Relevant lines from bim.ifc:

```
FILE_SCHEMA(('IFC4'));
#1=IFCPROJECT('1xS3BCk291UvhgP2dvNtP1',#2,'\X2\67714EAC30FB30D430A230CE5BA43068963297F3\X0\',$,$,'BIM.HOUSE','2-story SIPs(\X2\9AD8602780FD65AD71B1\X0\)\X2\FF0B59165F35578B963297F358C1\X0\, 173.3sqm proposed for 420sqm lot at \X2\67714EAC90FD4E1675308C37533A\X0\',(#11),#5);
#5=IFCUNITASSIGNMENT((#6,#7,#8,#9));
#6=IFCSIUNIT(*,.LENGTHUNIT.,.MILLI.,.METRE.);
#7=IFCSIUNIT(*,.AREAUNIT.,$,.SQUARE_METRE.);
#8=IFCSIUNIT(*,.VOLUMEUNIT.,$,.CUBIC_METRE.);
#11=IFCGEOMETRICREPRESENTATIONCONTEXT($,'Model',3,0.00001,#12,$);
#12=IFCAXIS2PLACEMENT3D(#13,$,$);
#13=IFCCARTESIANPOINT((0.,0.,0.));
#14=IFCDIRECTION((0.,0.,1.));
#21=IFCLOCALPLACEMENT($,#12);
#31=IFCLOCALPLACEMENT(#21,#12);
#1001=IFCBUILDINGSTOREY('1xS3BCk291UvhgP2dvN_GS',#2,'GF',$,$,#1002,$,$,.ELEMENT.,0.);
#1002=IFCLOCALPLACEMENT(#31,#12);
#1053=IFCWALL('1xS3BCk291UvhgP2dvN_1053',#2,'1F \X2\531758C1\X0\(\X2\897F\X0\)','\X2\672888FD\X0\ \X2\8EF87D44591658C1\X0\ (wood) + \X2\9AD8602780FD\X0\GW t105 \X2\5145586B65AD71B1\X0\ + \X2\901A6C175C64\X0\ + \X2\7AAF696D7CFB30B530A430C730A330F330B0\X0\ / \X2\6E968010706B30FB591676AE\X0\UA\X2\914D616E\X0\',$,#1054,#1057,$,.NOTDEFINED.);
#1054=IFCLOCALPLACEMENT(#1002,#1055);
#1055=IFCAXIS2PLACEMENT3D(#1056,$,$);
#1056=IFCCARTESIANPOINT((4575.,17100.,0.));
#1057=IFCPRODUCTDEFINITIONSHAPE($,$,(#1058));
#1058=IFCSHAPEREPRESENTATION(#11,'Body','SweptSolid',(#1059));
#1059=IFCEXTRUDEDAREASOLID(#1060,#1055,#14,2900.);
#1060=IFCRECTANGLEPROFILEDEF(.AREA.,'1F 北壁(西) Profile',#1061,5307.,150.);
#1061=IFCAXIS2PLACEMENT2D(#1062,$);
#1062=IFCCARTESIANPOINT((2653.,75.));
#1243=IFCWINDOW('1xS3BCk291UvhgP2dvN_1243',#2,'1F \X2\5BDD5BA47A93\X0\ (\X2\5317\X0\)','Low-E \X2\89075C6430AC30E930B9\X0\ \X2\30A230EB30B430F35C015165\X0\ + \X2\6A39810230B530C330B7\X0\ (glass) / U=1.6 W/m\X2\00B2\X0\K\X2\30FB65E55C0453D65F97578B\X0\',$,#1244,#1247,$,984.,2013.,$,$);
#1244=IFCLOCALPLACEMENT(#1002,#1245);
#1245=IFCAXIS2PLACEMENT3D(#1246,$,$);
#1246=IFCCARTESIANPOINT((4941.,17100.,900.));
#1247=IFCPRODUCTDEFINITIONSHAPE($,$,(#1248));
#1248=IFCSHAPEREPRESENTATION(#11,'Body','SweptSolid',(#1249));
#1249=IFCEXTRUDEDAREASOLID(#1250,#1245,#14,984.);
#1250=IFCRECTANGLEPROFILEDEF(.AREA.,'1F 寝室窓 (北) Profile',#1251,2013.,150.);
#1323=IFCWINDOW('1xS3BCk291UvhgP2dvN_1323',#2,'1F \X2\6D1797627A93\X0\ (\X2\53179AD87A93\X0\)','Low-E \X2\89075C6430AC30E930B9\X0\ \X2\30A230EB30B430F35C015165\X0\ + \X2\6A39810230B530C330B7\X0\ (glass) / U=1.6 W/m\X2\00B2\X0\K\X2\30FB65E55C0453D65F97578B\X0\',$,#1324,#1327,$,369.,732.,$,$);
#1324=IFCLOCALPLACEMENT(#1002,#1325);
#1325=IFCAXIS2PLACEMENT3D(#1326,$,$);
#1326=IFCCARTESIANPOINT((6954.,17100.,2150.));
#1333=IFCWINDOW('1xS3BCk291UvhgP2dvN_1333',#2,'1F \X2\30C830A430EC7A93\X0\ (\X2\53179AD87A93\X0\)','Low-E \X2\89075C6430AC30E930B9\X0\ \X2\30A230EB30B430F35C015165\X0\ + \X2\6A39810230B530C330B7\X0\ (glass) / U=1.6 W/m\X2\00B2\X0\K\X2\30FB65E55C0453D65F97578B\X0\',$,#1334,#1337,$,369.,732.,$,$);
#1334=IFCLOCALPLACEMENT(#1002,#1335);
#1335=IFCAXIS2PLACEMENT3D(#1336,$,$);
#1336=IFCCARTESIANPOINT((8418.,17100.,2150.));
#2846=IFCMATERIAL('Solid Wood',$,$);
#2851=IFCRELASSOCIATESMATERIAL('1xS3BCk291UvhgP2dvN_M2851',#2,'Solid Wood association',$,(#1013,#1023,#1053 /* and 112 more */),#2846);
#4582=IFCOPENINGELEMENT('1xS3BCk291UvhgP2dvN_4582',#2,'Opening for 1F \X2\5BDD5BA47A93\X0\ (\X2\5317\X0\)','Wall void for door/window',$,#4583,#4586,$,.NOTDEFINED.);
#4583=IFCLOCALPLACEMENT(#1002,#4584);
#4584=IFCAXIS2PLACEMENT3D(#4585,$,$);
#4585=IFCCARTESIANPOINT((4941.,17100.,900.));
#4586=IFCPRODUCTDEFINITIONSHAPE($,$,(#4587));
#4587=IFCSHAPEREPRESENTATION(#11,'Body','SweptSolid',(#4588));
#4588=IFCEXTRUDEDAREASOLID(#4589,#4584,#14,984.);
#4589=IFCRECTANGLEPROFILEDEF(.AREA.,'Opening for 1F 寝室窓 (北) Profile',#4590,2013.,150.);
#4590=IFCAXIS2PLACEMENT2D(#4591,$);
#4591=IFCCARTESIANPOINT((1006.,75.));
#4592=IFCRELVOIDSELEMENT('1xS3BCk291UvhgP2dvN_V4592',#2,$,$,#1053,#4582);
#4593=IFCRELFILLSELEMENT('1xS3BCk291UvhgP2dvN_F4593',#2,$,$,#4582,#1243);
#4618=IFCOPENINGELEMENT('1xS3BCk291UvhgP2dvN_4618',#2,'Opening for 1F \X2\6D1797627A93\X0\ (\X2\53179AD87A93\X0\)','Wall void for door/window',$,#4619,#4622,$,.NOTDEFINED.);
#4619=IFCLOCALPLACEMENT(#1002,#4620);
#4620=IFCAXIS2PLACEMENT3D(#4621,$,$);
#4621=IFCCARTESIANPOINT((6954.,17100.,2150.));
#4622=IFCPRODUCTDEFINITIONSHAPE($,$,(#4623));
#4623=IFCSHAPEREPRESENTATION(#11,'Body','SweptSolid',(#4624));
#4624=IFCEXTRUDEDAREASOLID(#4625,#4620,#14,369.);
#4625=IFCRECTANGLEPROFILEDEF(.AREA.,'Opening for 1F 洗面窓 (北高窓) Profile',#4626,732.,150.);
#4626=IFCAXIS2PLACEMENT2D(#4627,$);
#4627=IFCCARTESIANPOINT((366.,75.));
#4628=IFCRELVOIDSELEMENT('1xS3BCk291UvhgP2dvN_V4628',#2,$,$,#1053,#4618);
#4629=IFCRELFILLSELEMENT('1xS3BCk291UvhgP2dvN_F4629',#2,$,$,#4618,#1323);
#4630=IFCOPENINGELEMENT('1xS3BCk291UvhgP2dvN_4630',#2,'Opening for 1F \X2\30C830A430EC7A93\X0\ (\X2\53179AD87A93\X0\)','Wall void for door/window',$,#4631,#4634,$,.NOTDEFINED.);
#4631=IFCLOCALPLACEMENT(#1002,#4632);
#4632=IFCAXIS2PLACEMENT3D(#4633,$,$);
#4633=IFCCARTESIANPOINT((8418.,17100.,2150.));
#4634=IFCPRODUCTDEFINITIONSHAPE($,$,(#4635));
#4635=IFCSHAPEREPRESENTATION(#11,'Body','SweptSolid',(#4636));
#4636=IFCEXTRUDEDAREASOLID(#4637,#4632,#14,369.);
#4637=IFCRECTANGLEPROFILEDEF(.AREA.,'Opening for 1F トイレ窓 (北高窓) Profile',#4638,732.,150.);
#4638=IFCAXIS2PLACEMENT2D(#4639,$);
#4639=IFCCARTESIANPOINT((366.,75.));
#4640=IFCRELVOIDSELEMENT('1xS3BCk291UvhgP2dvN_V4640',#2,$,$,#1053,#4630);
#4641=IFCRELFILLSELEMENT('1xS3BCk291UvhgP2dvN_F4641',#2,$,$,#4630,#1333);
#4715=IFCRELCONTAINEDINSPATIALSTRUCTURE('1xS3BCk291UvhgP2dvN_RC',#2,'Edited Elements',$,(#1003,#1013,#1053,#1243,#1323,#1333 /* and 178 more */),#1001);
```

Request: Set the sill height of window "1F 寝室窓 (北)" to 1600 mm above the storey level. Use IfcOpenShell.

```python
import numpy as np
import ifcopenshell
import ifcopenshell.api.geometry
import ifcopenshell.geom
import ifcopenshell.util.element
import ifcopenshell.util.placement
import ifcopenshell.util.shape
import ifcopenshell.util.unit

model = ifcopenshell.open("bim.ifc")
unit_scale = ifcopenshell.util.unit.calculate_unit_scale(model)

window = model.by_guid("1xS3BCk291UvhgP2dvN_1243")
opening = window.FillsVoids[0].RelatingOpeningElement
storey = ifcopenshell.util.element.get_container(window, ifc_class="IfcBuildingStorey")
level = ifcopenshell.util.placement.get_local_placement(storey.ObjectPlacement)[2, 3]

# The opening's origin need not be at the sill, so measure its lowest point.
shape = ifcopenshell.geom.create_shape(ifcopenshell.geom.settings(), opening)
bottom = ifcopenshell.util.shape.get_shape_bottom_elevation(shape, shape.geometry) / unit_scale
dz = level + 1600.0 - bottom

shift = np.array([0.0, 0.0, dz])
# The window is not placed relative to its opening, so move both.
for product in (opening, window):
    matrix = ifcopenshell.util.placement.get_local_placement(product.ObjectPlacement)
    matrix[:3, 3] += shift
    ifcopenshell.api.geometry.edit_object_placement(model, product=product, matrix=matrix, is_si=False)

print(f"moved by {dz * unit_scale:+.3f} m")

model.write("bim_rev.ifc")
```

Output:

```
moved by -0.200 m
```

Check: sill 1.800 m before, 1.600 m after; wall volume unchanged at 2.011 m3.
